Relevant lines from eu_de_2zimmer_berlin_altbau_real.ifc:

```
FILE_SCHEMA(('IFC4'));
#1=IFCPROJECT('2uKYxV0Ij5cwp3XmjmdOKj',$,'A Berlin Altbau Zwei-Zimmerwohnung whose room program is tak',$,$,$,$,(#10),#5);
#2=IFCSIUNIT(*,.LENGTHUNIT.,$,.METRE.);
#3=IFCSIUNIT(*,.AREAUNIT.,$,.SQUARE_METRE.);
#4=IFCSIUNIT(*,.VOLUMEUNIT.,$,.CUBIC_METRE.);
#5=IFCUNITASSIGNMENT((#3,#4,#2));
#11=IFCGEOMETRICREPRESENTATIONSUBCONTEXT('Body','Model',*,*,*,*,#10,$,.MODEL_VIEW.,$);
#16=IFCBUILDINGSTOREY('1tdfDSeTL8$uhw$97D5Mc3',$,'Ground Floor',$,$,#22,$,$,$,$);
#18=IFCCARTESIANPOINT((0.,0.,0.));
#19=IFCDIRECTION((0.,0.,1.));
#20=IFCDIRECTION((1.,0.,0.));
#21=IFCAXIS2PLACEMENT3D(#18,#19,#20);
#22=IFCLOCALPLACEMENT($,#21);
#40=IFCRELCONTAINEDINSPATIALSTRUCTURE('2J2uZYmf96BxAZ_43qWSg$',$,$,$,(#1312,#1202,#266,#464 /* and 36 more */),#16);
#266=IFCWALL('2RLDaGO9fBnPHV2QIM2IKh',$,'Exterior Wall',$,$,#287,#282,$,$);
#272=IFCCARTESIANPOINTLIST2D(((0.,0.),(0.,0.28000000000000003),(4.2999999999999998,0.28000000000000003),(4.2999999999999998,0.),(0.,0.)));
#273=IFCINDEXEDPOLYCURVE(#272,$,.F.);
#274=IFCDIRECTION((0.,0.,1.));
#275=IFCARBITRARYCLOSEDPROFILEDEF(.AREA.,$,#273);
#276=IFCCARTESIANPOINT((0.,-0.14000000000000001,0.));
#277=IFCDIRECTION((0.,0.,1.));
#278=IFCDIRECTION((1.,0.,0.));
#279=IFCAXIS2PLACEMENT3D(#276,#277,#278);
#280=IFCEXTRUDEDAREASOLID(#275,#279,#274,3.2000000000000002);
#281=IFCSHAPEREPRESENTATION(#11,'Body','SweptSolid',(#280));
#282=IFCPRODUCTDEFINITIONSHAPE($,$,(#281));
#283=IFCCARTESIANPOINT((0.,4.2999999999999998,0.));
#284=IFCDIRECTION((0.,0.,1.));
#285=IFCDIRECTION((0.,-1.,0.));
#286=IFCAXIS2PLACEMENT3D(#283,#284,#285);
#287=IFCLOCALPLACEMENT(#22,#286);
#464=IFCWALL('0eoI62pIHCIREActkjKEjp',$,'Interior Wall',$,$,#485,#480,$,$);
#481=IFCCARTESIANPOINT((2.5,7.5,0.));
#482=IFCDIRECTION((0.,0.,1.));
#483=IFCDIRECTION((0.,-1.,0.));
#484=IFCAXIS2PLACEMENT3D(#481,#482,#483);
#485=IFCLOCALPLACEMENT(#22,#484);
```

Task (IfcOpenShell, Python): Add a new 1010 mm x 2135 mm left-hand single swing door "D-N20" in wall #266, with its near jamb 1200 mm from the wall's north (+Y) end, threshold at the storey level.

```python
import numpy as np
import ifcopenshell
import ifcopenshell.api.feature
import ifcopenshell.api.geometry
import ifcopenshell.api.root
import ifcopenshell.api.spatial
import ifcopenshell.geom
import ifcopenshell.util.element
import ifcopenshell.util.placement
import ifcopenshell.util.representation
import ifcopenshell.util.shape
import ifcopenshell.util.unit

model = ifcopenshell.open("eu_de_2zimmer_berlin_altbau_real.ifc")
unit_scale = ifcopenshell.util.unit.calculate_unit_scale(model)
settings = ifcopenshell.geom.settings()


def volume(element):
    """Net volume in cubic metres, openings subtracted."""
    shape = ifcopenshell.geom.create_shape(settings, element)
    return ifcopenshell.util.shape.get_volume(shape.geometry)


wall = model.by_guid("2RLDaGO9fBnPHV2QIM2IKh")
storey = ifcopenshell.util.element.get_container(wall, ifc_class="IfcBuildingStorey")
context = ifcopenshell.util.representation.get_context(model, "Model", "Body", "MODEL_VIEW")
before = volume(wall)

width, height, from_end, sill = 1.01, 2.135, 1.2, 0.0  # metres

# The wall runs along its own X axis, and the end named is its -X end.
wall_shape = ifcopenshell.geom.create_shape(settings, wall)
x, y, z = ifcopenshell.util.shape.get_vertices(wall_shape.geometry).T
start = x.min() + from_end
face, thickness = float(y.min()), float(y.max() - y.min())
wall_matrix = ifcopenshell.util.placement.get_local_placement(wall.ObjectPlacement)
level = ifcopenshell.util.placement.get_local_placement(storey.ObjectPlacement)[2, 3]


def in_wall(x, y):
    """Placement at x, y metres in the wall's axes, at sill height."""
    matrix = wall_matrix.copy()
    matrix[:, 3] = wall_matrix @ np.array([x / unit_scale, y / unit_scale, 0.0, 1.0])
    matrix[2, 3] = level + sill / unit_scale
    return matrix


# Opening: a box that overshoots both wall faces by 50 mm.
opening = ifcopenshell.api.root.create_entity(model, ifc_class="IfcOpeningElement", predefined_type="OPENING")
box = ifcopenshell.api.geometry.add_wall_representation(
    model, context=context, length=width, height=height, thickness=thickness + 0.1
)
ifcopenshell.api.geometry.assign_representation(model, product=opening, representation=box)
ifcopenshell.api.geometry.edit_object_placement(model, product=opening, matrix=in_wall(start, face - 0.05), is_si=False)
ifcopenshell.api.feature.add_feature(model, feature=opening, element=wall)

door = ifcopenshell.api.root.create_entity(model, ifc_class="IfcDoor", name="D-N20", predefined_type="DOOR")
door.OverallWidth, door.OverallHeight = width / unit_scale, height / unit_scale
door.OperationType = "SINGLE_SWING_LEFT"
body = ifcopenshell.api.geometry.add_door_representation(
    model,
    context=context,
    overall_width=door.OverallWidth,
    overall_height=door.OverallHeight,
    operation_type="SINGLE_SWING_LEFT",
    lining_properties={"LiningDepth": thickness / unit_scale, "ThresholdDepth": thickness / unit_scale},
)
ifcopenshell.api.geometry.assign_representation(model, product=door, representation=body)
ifcopenshell.api.spatial.assign_container(model, products=[door], relating_structure=storey)
ifcopenshell.api.feature.add_filling(model, opening=opening, element=door)

# The lining spans the wall, so the door starts at the wall face.
ifcopenshell.api.geometry.edit_object_placement(model, product=door, matrix=in_wall(start, face), is_si=False)

after = volume(wall)

print(f"wall volume {before:.3f} -> {after:.3f} m3")

model.write("eu_de_2zimmer_berlin_altbau_real_v2.ifc")
```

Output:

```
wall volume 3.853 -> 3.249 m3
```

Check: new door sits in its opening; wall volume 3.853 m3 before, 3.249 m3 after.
